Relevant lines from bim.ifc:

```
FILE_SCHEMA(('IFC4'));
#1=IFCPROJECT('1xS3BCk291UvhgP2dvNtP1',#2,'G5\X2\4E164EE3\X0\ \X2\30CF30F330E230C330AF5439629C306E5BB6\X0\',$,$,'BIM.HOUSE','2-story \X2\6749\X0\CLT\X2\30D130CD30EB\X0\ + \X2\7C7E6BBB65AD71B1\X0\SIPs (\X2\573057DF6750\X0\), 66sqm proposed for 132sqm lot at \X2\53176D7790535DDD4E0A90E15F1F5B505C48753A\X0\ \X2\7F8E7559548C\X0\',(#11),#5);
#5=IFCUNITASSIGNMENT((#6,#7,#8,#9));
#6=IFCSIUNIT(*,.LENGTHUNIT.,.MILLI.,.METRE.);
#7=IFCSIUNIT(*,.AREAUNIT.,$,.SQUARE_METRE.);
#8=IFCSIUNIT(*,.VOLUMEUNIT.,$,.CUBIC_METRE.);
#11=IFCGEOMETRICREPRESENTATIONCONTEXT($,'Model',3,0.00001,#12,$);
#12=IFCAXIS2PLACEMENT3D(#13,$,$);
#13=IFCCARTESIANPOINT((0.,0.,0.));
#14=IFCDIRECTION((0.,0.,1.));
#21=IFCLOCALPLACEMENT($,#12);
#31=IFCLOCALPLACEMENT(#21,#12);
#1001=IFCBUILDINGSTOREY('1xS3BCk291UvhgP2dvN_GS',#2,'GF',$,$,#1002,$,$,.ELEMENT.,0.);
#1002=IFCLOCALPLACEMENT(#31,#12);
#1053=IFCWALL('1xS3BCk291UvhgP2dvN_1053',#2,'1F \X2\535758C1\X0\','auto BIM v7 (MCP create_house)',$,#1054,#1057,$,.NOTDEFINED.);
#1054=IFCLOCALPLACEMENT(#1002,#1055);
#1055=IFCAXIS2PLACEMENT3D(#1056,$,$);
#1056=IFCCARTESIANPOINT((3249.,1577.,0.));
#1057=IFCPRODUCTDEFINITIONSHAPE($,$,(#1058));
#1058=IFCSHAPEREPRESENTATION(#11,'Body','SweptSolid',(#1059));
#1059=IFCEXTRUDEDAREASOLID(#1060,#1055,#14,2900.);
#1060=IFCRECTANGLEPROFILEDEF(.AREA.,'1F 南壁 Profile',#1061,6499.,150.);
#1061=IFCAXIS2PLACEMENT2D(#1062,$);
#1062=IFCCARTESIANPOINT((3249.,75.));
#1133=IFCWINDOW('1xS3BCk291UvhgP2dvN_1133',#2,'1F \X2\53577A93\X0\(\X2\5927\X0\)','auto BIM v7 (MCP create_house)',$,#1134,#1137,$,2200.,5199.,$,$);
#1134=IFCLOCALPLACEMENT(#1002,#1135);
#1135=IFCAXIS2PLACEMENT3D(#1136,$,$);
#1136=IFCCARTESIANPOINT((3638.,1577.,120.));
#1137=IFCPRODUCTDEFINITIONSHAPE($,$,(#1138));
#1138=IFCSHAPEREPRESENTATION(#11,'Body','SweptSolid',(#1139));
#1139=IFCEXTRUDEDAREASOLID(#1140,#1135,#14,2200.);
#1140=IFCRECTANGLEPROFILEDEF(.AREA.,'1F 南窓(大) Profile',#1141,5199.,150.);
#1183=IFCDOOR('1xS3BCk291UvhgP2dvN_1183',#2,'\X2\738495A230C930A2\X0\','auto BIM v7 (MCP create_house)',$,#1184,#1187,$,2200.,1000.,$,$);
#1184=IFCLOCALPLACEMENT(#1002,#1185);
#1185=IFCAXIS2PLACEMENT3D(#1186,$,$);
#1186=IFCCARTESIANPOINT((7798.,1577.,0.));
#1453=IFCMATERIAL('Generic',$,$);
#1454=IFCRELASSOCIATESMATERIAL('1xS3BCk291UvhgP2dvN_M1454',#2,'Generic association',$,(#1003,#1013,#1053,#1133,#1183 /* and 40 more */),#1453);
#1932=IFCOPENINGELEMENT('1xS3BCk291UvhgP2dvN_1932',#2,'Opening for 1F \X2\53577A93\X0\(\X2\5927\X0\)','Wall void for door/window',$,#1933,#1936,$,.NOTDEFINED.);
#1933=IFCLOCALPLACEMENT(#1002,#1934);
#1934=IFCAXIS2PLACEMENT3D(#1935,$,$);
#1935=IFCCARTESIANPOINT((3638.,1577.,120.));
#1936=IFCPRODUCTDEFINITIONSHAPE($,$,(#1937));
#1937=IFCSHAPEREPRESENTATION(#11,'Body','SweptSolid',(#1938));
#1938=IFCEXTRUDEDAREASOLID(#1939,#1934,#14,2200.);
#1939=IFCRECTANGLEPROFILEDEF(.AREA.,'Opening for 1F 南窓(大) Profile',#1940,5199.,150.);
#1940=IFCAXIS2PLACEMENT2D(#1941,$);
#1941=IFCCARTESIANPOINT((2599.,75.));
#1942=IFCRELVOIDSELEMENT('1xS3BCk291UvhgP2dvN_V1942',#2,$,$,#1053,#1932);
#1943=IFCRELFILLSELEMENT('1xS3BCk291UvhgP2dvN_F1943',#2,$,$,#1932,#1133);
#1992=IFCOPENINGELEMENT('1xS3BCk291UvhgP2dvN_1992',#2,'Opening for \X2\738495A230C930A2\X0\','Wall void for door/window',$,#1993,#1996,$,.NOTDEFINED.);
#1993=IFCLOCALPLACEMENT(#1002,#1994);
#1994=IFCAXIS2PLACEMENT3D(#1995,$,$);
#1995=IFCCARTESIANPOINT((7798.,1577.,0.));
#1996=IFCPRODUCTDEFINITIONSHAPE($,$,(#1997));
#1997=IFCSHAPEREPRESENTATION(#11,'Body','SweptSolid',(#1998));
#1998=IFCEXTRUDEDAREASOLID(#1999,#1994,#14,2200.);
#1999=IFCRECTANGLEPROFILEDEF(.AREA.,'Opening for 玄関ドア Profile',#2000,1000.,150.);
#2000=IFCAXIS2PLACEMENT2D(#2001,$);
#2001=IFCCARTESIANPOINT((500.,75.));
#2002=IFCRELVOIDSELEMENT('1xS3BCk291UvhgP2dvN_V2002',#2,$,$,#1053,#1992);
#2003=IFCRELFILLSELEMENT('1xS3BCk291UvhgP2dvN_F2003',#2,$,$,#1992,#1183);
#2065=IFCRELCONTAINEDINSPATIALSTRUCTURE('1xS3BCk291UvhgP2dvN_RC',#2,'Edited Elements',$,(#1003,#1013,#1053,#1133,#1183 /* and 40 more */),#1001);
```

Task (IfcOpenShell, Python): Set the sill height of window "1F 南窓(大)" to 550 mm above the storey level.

```python
import numpy as np
import ifcopenshell
import ifcopenshell.api.geometry
import ifcopenshell.geom
import ifcopenshell.util.element
import ifcopenshell.util.placement
import ifcopenshell.util.shape
import ifcopenshell.util.unit

model = ifcopenshell.open("bim.ifc")
unit_scale = ifcopenshell.util.unit.calculate_unit_scale(model)

window = model.by_guid("1xS3BCk291UvhgP2dvN_1133")
opening = window.FillsVoids[0].RelatingOpeningElement
storey = ifcopenshell.util.element.get_container(window, ifc_class="IfcBuildingStorey")
level = ifcopenshell.util.placement.get_local_placement(storey.ObjectPlacement)[2, 3]

# The opening's origin need not be at the sill, so measure its lowest point.
shape = ifcopenshell.geom.create_shape(ifcopenshell.geom.settings(), opening)
bottom = ifcopenshell.util.shape.get_shape_bottom_elevation(shape, shape.geometry) / unit_scale
dz = level + 0.55 / unit_scale - bottom

shift = np.array([0.0, 0.0, dz])
# The window is not placed relative to its opening, so move both.
for product in (opening, window):
    matrix = ifcopenshell.util.placement.get_local_placement(product.ObjectPlacement)
    matrix[:3, 3] += shift
    ifcopenshell.api.geometry.edit_object_placement(model, product=product, matrix=matrix, is_si=False)

print(f"moved by {dz * unit_scale:+.3f} m")

model.write("bim-out.ifc")
```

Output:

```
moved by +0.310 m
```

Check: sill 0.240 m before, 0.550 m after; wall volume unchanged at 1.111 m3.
